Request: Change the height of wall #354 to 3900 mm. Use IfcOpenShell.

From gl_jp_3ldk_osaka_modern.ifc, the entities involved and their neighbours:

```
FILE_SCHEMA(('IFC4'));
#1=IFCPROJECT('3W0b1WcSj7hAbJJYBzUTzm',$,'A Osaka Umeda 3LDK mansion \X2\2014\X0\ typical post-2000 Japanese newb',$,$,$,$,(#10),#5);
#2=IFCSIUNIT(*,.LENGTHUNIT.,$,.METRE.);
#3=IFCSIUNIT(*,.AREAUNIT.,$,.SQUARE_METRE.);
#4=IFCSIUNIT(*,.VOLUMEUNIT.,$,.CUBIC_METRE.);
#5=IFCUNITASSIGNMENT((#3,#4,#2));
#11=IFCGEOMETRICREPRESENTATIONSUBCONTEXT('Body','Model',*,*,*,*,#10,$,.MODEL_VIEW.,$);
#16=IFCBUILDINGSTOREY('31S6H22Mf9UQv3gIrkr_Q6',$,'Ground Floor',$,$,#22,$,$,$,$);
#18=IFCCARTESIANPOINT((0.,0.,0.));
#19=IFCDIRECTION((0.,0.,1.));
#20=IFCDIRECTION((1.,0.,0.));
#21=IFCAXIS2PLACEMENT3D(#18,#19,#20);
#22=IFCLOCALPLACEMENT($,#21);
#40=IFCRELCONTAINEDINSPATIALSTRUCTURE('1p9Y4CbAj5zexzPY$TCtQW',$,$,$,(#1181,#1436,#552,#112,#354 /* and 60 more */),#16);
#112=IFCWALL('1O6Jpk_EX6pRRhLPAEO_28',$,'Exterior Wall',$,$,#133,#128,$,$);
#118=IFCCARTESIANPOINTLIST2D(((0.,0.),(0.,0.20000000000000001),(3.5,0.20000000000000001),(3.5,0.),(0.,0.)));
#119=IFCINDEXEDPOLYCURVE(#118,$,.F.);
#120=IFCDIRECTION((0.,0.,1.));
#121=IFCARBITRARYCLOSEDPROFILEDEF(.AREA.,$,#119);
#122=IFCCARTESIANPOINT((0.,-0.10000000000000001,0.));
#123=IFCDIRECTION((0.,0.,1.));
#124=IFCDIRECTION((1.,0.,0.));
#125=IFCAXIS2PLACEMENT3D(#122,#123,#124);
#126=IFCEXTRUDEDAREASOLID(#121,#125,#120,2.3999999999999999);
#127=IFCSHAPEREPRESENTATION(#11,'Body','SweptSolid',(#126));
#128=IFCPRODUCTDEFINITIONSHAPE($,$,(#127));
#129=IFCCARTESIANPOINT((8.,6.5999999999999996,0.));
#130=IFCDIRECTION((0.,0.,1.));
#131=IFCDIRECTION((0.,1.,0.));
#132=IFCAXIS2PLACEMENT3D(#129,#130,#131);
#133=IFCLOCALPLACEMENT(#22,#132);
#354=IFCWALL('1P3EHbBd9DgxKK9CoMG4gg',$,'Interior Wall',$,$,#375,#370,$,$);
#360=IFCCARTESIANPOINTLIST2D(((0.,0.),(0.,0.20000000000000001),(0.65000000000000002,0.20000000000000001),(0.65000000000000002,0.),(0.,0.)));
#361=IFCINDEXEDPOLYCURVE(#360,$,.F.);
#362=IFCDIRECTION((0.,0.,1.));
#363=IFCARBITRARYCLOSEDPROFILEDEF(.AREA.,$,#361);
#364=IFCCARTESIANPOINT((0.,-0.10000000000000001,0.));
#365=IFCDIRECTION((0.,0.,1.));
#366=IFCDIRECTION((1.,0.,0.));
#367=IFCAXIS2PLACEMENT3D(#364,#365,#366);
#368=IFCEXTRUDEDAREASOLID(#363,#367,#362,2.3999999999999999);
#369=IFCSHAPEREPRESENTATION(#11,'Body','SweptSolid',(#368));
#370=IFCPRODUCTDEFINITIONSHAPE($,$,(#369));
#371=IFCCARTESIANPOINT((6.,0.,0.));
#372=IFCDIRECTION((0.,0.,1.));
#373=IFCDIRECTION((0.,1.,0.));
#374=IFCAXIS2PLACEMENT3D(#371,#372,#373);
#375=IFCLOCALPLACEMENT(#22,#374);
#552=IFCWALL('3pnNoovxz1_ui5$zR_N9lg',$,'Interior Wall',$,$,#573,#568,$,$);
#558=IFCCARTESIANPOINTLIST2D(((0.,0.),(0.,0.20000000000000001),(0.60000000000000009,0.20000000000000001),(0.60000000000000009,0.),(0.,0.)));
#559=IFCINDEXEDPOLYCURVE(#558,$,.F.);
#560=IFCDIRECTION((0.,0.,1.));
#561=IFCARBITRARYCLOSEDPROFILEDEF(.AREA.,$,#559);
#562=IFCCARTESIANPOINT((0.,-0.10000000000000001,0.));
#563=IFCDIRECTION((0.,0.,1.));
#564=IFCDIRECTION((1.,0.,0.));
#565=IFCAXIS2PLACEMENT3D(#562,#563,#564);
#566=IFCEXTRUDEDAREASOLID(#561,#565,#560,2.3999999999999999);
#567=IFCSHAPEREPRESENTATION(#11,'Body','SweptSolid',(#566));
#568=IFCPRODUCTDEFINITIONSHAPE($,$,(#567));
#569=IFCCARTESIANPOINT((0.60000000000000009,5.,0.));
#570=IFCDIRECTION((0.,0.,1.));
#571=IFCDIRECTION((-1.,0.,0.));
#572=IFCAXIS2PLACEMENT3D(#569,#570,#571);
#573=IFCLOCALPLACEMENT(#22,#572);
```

```python
import ifcopenshell
import ifcopenshell.geom
import ifcopenshell.util.representation
import ifcopenshell.util.shape
import ifcopenshell.util.unit

model = ifcopenshell.open("gl_jp_3ldk_osaka_modern.ifc")
unit_scale = ifcopenshell.util.unit.calculate_unit_scale(model)
settings = ifcopenshell.geom.settings()


def volume(element):
    """Net volume in cubic metres, openings subtracted."""
    shape = ifcopenshell.geom.create_shape(settings, element)
    return ifcopenshell.util.shape.get_volume(shape.geometry)


wall = model.by_id(354)
before = volume(wall)

body = ifcopenshell.util.representation.get_representation(wall, "Model", "Body")
solid = body.Items[0]
old_height = solid.Depth
solid.Depth = 3.9 / unit_scale
after = volume(wall)

print(f"height {old_height:g} -> {solid.Depth:g}, volume {before:.3f} -> {after:.3f} m3")

model.write("gl_jp_3ldk_osaka_modern-out.ifc")
```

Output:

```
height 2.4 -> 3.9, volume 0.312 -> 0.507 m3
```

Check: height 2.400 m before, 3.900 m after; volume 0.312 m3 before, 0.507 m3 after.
